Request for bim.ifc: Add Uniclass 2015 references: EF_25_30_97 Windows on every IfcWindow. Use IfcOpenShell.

First a look at what the model holds.

```python
import ifcopenshell

model = ifcopenshell.open("bim.ifc")
print(model.schema)
print("classifications:", [c.Name for c in model.by_type("IfcClassification")])
for ifc_class in ("IfcDoor", "IfcRoof", "IfcStair", "IfcWall", "IfcWindow"):
    print(ifc_class, len(model.by_type(ifc_class)))
```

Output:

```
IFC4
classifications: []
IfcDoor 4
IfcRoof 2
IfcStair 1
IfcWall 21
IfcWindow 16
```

```python
import ifcopenshell
import ifcopenshell.api.classification

model = ifcopenshell.open("bim.ifc")

system = ifcopenshell.api.classification.add_classification(model, classification="Uniclass 2015")

codes = {
    "IfcWindow": ("EF_25_30_97", "Windows"),
}
for ifc_class, (code, name) in codes.items():
    products = model.by_type(ifc_class)
    ifcopenshell.api.classification.add_reference(
        model, products=products, classification=system, identification=code, name=name
    )
    print(code, len(products))

model.write("bim-out.ifc")
```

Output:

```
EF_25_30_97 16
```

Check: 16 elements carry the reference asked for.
